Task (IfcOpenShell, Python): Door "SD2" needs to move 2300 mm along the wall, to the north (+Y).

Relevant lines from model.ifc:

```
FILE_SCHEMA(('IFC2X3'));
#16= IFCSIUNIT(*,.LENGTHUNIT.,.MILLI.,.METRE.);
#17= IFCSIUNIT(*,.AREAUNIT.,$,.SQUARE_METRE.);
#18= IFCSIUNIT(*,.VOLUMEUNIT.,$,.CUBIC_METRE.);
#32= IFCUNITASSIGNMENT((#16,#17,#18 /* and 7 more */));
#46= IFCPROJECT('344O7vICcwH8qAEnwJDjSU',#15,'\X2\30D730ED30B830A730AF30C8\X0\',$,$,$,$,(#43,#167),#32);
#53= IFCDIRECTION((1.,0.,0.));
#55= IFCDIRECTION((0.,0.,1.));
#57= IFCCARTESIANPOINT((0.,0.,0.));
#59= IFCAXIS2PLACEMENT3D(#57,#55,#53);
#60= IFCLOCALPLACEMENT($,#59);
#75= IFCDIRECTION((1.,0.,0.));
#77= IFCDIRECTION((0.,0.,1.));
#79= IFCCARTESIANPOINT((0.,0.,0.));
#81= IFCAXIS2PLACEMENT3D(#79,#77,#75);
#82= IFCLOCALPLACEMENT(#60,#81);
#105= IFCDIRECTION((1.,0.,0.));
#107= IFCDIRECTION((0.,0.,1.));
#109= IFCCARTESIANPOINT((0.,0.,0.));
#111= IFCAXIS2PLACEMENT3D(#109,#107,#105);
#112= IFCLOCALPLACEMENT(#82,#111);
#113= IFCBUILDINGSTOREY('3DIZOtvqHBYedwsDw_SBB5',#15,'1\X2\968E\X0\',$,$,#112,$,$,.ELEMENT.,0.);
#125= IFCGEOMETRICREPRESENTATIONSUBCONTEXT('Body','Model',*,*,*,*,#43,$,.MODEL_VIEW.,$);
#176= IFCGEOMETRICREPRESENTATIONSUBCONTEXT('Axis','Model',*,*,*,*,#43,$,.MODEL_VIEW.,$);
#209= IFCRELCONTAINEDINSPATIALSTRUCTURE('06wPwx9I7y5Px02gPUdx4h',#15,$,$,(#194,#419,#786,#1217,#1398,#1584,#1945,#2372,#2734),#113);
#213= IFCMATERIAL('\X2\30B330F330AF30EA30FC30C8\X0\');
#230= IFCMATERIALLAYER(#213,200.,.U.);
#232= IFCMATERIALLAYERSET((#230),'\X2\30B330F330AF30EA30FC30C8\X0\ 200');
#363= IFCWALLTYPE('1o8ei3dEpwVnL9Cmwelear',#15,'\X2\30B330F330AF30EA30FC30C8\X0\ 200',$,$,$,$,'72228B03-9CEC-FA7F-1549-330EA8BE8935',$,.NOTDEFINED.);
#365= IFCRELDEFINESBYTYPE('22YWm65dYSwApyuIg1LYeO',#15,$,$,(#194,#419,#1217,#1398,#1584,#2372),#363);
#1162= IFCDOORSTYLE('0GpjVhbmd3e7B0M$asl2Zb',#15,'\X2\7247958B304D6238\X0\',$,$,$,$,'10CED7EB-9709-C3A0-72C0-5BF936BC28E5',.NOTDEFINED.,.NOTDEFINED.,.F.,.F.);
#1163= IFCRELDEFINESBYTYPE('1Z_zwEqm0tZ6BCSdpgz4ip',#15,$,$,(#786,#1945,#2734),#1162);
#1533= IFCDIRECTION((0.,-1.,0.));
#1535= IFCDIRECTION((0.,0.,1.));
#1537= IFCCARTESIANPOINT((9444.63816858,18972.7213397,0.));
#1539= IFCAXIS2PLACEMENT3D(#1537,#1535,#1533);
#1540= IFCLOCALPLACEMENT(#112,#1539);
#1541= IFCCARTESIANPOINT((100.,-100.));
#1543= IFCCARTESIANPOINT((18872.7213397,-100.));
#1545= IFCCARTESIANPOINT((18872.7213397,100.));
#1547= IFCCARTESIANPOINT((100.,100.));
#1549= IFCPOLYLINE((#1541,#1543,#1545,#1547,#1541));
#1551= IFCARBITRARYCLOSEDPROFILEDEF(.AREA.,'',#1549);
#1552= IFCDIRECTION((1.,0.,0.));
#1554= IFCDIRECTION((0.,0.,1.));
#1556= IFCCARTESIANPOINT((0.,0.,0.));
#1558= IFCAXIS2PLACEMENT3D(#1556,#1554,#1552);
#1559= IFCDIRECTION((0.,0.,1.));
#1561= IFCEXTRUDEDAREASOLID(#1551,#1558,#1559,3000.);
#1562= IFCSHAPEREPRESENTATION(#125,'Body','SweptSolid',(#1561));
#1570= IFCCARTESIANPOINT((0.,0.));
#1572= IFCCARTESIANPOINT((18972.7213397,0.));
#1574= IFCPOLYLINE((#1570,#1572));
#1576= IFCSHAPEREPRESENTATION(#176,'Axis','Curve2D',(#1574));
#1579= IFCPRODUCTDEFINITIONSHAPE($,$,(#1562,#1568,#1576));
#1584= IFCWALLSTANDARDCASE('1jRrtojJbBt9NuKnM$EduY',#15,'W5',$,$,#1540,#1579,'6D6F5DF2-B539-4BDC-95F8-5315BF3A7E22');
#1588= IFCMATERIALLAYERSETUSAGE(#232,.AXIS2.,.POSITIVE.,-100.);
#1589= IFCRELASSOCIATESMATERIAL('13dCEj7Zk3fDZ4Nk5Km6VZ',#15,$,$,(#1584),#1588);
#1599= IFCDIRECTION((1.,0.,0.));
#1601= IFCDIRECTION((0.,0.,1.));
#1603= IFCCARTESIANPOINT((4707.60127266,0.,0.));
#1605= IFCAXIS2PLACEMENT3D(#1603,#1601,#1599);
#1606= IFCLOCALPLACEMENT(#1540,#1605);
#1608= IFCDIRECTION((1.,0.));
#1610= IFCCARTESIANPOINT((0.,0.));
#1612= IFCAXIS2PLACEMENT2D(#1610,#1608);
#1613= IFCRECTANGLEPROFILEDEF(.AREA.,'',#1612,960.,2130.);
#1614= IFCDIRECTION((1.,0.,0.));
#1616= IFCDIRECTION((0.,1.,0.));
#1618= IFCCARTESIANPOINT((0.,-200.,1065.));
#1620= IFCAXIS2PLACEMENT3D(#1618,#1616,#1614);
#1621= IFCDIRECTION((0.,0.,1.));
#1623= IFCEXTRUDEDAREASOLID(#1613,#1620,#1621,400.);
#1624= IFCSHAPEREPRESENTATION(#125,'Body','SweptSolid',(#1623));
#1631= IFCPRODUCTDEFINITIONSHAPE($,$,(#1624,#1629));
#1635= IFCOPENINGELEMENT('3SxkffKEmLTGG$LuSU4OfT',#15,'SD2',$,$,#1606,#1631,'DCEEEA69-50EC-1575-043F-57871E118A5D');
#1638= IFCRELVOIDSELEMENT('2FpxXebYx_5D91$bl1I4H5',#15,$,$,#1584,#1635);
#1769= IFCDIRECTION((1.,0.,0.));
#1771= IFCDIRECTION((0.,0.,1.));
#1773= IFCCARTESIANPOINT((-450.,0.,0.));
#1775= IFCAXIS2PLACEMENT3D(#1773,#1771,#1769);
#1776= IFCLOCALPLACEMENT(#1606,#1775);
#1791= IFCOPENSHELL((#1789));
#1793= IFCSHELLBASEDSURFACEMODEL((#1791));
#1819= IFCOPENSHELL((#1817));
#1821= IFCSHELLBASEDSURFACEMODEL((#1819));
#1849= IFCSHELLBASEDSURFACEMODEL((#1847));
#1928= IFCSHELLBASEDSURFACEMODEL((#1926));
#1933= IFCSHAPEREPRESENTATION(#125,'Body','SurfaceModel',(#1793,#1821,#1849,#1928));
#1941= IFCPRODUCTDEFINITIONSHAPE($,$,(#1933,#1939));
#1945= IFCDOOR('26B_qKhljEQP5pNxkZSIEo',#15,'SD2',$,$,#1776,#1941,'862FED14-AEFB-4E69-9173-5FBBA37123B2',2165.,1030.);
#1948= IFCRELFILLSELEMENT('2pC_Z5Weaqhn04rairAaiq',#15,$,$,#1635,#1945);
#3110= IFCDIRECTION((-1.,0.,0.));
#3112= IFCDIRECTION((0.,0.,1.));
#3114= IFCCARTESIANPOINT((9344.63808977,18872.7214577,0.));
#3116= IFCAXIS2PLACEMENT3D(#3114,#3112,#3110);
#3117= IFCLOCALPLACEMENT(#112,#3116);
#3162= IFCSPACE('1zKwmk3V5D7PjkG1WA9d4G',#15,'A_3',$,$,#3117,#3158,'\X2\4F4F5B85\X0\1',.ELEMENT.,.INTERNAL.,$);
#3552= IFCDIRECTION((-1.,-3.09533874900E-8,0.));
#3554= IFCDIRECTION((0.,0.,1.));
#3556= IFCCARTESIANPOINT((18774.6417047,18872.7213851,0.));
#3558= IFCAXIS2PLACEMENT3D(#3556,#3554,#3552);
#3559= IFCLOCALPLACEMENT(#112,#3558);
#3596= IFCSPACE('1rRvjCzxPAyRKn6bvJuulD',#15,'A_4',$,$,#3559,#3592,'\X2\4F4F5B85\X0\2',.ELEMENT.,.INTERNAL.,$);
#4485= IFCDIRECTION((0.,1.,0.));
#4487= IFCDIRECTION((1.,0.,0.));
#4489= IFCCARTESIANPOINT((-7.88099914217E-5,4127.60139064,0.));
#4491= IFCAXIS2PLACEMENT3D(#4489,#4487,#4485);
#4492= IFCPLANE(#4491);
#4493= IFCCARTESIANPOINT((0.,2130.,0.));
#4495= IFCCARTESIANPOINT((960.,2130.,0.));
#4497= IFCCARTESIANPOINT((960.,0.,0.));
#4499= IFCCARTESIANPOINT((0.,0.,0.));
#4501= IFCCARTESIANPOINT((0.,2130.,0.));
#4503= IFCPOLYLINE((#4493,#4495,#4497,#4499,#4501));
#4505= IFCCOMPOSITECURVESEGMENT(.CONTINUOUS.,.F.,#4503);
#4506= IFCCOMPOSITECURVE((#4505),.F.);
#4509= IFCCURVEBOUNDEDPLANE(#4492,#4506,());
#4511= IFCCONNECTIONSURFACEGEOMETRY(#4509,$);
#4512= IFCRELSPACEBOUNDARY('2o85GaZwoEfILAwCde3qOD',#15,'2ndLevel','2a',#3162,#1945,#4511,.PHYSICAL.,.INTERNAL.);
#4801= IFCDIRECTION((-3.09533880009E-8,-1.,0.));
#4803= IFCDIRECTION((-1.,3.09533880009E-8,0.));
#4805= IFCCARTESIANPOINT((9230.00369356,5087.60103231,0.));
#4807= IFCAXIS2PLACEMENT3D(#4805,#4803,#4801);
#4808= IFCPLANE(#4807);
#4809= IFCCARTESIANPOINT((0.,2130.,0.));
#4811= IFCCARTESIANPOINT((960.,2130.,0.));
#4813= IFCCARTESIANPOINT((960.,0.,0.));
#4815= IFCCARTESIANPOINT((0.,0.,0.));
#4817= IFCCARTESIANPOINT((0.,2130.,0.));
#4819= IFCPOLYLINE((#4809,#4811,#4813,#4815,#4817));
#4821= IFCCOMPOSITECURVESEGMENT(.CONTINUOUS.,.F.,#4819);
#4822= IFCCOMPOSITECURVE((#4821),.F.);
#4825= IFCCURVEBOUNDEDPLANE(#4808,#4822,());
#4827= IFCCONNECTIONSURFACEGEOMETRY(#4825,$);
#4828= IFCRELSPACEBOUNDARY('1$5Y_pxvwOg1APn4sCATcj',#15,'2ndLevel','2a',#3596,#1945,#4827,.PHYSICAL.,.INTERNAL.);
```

```python
import numpy as np
import ifcopenshell
import ifcopenshell.api.geometry
import ifcopenshell.util.placement
import ifcopenshell.util.unit

model = ifcopenshell.open("model.ifc")
unit_scale = ifcopenshell.util.unit.calculate_unit_scale(model)

door = model.by_guid("26B_qKhljEQP5pNxkZSIEo")
opening = door.FillsVoids[0].RelatingOpeningElement
wall = opening.VoidsElements[0].RelatingBuildingElement

wall_matrix = ifcopenshell.util.placement.get_local_placement(wall.ObjectPlacement)
shift = wall_matrix[:3, 0] * -2.3 / unit_scale
before = ifcopenshell.util.placement.get_local_placement(door.ObjectPlacement)[:3, 3].copy()

# The door is placed relative to its opening, so it follows when the opening moves.
matrix = ifcopenshell.util.placement.get_local_placement(opening.ObjectPlacement)
matrix[:3, 3] += shift
ifcopenshell.api.geometry.edit_object_placement(
    model, product=opening, matrix=matrix, is_si=False, should_transform_children=True
)

# Space boundary surfaces are stored in each space's coordinates; move them too.
for rel in door.ProvidesBoundaries:
    if not rel.ConnectionGeometry:
        continue
    surface = rel.ConnectionGeometry.SurfaceOnRelatingElement.BasisSurface
    space_matrix = ifcopenshell.util.placement.get_local_placement(rel.RelatingSpace.ObjectPlacement)
    point = np.array(surface.Position.Location.Coordinates) + space_matrix[:3, :3].T @ shift
    surface.Position = model.createIfcAxis2Placement3D(
        model.createIfcCartesianPoint(point.tolist()), surface.Position.Axis, surface.Position.RefDirection
    )

after = ifcopenshell.util.placement.get_local_placement(door.ObjectPlacement)[:3, 3]
print("door moved by", (after - before).round(3) + 0.0)

model.write("model_rev.ifc")
```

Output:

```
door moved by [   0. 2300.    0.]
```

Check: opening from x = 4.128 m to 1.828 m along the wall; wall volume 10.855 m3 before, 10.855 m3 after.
